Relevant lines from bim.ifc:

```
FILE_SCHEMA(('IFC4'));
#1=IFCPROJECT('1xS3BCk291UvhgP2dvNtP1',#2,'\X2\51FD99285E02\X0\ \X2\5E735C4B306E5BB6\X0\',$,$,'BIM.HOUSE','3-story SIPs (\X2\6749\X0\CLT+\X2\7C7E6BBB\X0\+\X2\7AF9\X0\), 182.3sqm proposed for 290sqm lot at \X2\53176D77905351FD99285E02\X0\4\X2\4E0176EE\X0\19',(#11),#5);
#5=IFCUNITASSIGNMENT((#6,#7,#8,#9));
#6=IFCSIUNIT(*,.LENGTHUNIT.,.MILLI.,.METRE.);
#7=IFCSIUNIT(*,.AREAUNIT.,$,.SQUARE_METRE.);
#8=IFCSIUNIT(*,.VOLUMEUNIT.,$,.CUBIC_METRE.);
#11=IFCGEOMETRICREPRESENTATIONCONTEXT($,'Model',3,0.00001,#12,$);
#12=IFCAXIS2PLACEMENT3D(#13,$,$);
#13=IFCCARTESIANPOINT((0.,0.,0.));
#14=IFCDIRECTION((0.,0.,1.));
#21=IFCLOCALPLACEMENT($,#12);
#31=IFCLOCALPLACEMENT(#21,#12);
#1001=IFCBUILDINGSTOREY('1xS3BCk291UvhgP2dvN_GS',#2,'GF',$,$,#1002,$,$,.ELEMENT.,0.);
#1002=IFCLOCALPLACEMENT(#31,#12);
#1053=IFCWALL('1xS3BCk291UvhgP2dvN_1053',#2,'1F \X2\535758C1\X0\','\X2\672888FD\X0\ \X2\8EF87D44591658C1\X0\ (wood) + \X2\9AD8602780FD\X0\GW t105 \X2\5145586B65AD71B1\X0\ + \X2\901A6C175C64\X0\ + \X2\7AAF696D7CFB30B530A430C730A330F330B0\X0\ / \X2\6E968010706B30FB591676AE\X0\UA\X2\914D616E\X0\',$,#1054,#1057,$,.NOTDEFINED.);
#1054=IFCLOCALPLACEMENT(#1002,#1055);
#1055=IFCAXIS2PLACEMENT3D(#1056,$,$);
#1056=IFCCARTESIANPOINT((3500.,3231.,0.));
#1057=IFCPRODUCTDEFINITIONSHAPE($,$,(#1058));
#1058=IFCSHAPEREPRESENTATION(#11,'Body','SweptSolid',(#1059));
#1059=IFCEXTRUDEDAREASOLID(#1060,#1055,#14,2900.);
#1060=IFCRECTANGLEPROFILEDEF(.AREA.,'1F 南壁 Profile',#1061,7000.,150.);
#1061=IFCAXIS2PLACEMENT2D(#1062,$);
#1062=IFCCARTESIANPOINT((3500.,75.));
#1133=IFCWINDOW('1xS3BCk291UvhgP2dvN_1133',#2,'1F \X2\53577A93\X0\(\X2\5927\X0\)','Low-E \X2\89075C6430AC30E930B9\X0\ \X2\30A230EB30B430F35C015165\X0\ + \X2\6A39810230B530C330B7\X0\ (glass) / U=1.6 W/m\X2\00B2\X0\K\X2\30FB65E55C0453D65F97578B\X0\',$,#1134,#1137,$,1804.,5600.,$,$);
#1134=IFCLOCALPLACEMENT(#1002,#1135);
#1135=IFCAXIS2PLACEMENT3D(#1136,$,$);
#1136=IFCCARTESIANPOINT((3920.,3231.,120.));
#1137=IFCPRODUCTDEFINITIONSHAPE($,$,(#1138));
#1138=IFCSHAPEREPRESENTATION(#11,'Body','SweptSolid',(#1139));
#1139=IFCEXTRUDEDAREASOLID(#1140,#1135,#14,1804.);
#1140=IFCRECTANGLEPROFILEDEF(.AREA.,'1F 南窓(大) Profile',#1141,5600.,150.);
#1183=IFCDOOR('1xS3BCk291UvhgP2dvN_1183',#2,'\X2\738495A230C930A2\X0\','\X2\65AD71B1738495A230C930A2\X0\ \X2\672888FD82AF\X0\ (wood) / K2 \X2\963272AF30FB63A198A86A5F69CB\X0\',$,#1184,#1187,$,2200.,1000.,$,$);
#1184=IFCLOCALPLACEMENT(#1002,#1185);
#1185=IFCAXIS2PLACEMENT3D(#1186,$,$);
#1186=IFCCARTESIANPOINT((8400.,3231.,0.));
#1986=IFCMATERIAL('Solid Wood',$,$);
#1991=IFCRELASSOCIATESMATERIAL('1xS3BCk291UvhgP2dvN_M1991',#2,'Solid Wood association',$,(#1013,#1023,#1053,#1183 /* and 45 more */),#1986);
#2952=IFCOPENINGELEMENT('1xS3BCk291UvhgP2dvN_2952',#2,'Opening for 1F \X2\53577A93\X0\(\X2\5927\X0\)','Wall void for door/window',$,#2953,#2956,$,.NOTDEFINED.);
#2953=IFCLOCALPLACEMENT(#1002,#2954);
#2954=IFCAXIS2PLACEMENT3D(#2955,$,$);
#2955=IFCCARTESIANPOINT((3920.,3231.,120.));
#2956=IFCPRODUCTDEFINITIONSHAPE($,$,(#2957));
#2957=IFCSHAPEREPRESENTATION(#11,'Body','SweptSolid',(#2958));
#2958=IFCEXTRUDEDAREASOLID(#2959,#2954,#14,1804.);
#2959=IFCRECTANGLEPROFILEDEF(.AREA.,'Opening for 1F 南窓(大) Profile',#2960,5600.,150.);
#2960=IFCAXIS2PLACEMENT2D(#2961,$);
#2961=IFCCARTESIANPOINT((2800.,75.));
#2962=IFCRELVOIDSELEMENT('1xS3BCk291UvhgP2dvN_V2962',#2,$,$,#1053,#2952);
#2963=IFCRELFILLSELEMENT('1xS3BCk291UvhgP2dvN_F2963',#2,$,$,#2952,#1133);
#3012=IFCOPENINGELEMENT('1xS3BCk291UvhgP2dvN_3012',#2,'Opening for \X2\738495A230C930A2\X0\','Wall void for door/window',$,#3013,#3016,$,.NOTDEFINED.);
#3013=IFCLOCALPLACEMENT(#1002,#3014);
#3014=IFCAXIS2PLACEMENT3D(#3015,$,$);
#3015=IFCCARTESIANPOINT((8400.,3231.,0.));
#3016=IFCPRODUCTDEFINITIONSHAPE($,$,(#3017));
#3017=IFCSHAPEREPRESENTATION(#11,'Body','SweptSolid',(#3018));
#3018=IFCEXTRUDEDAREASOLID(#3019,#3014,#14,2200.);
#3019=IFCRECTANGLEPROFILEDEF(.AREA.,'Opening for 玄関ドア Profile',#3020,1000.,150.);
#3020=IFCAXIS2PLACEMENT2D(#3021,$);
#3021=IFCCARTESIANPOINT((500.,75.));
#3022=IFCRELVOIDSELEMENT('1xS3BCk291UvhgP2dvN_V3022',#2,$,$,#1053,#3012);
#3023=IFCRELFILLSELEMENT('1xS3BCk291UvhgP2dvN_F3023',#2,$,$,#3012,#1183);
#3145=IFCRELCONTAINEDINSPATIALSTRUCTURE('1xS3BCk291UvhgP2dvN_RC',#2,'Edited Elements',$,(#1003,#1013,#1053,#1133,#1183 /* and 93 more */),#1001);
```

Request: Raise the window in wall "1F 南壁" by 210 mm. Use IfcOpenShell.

```python
import numpy as np
import ifcopenshell
import ifcopenshell.api.geometry
import ifcopenshell.util.placement
import ifcopenshell.util.unit

model = ifcopenshell.open("bim.ifc")
unit_scale = ifcopenshell.util.unit.calculate_unit_scale(model)

window = model.by_guid("1xS3BCk291UvhgP2dvN_1133")
opening = window.FillsVoids[0].RelatingOpeningElement
dz = 210.0

shift = np.array([0.0, 0.0, dz])
# The window is not placed relative to its opening, so move both.
for product in (opening, window):
    matrix = ifcopenshell.util.placement.get_local_placement(product.ObjectPlacement)
    matrix[:3, 3] += shift
    ifcopenshell.api.geometry.edit_object_placement(model, product=product, matrix=matrix, is_si=False)

print(f"moved by {dz * unit_scale:+.3f} m")

model.write("bim_updated.ifc")
```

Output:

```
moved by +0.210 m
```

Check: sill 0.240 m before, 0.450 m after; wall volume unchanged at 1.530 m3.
